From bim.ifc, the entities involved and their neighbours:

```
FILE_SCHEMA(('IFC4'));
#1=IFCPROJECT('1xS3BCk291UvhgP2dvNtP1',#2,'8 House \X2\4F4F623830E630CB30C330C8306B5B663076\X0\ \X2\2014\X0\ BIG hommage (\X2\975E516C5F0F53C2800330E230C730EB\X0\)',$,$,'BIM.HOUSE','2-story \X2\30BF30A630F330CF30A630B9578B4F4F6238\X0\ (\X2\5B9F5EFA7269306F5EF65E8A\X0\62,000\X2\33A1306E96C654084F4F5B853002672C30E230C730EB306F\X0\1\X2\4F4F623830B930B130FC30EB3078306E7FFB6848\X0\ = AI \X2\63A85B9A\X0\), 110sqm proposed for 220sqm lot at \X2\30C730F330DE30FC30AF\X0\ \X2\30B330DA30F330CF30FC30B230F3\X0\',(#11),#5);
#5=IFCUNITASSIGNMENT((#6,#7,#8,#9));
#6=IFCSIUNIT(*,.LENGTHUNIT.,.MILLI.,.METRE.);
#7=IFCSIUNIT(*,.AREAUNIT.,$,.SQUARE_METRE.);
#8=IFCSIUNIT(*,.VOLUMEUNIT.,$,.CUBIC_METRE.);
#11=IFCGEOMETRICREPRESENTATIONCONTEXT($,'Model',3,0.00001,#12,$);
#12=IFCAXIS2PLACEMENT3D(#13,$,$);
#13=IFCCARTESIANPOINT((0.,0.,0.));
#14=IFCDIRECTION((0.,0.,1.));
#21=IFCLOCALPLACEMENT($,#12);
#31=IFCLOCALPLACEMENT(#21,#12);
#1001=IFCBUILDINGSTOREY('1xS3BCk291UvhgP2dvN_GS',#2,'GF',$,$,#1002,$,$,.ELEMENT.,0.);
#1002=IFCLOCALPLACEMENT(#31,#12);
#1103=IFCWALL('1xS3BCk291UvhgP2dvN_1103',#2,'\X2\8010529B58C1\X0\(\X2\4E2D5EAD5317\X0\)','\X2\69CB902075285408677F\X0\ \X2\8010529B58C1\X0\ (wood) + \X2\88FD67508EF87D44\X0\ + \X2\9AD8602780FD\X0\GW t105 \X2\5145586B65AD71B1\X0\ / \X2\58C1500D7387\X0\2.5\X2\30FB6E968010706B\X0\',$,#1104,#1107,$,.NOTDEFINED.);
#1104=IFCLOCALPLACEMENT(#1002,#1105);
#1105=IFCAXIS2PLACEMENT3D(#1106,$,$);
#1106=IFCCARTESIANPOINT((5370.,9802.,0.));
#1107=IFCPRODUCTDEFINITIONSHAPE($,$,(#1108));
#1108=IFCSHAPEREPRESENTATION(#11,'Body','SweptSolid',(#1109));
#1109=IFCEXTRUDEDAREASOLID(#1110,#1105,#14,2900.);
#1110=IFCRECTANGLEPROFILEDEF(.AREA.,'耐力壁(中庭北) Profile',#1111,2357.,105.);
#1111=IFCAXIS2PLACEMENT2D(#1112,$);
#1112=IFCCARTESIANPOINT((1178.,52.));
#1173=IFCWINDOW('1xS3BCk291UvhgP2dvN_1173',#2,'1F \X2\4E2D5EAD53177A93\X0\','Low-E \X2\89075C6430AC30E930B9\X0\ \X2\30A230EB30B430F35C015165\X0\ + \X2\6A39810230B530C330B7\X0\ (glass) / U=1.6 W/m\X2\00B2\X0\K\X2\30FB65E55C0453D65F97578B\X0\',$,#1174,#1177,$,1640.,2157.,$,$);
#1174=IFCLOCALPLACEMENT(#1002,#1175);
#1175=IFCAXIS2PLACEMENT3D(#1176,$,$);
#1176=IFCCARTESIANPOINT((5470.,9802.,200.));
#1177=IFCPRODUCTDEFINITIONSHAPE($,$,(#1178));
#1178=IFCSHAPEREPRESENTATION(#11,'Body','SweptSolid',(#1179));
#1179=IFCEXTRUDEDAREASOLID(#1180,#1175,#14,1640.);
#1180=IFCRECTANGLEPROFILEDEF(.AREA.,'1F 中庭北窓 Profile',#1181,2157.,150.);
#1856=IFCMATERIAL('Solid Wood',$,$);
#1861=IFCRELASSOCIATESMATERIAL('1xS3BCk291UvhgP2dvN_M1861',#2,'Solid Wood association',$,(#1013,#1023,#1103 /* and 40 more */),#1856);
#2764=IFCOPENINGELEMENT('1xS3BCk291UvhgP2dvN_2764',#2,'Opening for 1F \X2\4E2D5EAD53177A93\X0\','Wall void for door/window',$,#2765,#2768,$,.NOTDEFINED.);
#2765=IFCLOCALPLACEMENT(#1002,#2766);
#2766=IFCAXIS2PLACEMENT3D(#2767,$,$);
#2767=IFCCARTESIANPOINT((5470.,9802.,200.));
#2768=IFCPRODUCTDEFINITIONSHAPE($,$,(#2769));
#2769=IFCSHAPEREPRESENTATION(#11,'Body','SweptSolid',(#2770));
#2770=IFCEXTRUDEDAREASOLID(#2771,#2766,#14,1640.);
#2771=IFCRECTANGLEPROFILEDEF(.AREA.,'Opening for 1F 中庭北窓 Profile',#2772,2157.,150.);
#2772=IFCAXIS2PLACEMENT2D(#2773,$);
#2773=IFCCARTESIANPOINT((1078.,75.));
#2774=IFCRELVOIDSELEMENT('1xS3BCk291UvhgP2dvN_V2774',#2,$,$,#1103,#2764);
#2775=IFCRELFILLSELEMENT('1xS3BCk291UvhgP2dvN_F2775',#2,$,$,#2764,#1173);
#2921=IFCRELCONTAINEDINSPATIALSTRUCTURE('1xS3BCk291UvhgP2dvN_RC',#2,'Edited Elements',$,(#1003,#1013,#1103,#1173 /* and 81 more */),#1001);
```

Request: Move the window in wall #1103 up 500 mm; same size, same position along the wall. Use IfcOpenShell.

```python
import numpy as np
import ifcopenshell
import ifcopenshell.api.geometry
import ifcopenshell.util.placement
import ifcopenshell.util.unit

model = ifcopenshell.open("bim.ifc")
unit_scale = ifcopenshell.util.unit.calculate_unit_scale(model)

window = model.by_guid("1xS3BCk291UvhgP2dvN_1173")
opening = window.FillsVoids[0].RelatingOpeningElement
dz = 0.5 / unit_scale

shift = np.array([0.0, 0.0, dz])
# The window is not placed relative to its opening, so move both.
for product in (opening, window):
    matrix = ifcopenshell.util.placement.get_local_placement(product.ObjectPlacement)
    matrix[:3, 3] += shift
    ifcopenshell.api.geometry.edit_object_placement(model, product=product, matrix=matrix, is_si=False)

print(f"moved by {dz * unit_scale:+.3f} m")

model.write("bim_v2.ifc")
```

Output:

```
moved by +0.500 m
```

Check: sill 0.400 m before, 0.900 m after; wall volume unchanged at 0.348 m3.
